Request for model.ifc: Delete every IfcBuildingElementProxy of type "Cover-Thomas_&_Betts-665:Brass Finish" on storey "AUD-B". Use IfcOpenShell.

First a look at what the model holds.

```python
import ifcopenshell
import ifcopenshell.util.element

model = ifcopenshell.open("model.ifc")
print(model.schema)
storey = next(s for s in model.by_type("IfcBuildingStorey") if s.Name == "AUD-B")
proxies = [e for e in ifcopenshell.util.element.get_decomposition(storey) if e.is_a("IfcBuildingElementProxy")]
seen = {}
for e in proxies:
    element_type = ifcopenshell.util.element.get_type(e)
    name = element_type.Name if element_type not in (None, e) else None
    seen[name] = seen.get(name, 0) + 1
for name, count in sorted(seen.items(), key=str):
    print(count, "x", name)
```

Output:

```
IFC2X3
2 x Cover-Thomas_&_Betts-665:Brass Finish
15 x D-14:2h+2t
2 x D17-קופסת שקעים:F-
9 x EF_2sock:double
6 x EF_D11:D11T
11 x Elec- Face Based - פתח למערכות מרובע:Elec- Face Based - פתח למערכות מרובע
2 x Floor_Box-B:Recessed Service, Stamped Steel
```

```python
import ifcopenshell
import ifcopenshell.api.root
import ifcopenshell.util.element

model = ifcopenshell.open("model.ifc")

storey = next(s for s in model.by_type("IfcBuildingStorey") if s.Name == "AUD-B")
proxies = [e for e in ifcopenshell.util.element.get_decomposition(storey) if e.is_a("IfcBuildingElementProxy")]
targets = [e for e in proxies if (t := ifcopenshell.util.element.get_type(e)) not in (None, e) and t.Name == "Cover-Thomas_&_Betts-665:Brass Finish"]

for e in targets:
    ifcopenshell.api.root.remove_product(model, product=e)
print(len(targets), "removed")

model.write("model_edited.ifc")
```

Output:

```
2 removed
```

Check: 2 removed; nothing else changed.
